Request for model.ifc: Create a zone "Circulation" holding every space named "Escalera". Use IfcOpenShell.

First a look at what the model holds.

```python
import ifcopenshell

model = ifcopenshell.open("model.ifc")
print(model.schema)
seen = {}
for space in model.by_type("IfcSpace"):
    seen[space.LongName] = seen.get(space.LongName, 0) + 1
for name, count in sorted(seen.items(), key=str):
    print(count, "x", name)
print("zones:", [z.Name for z in model.by_type("IfcZone")][:20])
```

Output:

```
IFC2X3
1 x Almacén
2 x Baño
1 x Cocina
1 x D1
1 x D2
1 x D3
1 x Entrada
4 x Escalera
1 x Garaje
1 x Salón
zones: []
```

```python
import ifcopenshell
import ifcopenshell.api.group
import ifcopenshell.api.root

model = ifcopenshell.open("model.ifc")

names = {"Escalera"}
spaces = [s for s in model.by_type("IfcSpace") if s.LongName in names]

zone = ifcopenshell.api.root.create_entity(model, ifc_class="IfcZone", name="Circulation")
ifcopenshell.api.group.assign_group(model, products=spaces, group=zone)
print(len(spaces), "spaces in", zone.Name)

model.write("model_updated.ifc")
```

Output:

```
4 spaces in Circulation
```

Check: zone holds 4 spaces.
